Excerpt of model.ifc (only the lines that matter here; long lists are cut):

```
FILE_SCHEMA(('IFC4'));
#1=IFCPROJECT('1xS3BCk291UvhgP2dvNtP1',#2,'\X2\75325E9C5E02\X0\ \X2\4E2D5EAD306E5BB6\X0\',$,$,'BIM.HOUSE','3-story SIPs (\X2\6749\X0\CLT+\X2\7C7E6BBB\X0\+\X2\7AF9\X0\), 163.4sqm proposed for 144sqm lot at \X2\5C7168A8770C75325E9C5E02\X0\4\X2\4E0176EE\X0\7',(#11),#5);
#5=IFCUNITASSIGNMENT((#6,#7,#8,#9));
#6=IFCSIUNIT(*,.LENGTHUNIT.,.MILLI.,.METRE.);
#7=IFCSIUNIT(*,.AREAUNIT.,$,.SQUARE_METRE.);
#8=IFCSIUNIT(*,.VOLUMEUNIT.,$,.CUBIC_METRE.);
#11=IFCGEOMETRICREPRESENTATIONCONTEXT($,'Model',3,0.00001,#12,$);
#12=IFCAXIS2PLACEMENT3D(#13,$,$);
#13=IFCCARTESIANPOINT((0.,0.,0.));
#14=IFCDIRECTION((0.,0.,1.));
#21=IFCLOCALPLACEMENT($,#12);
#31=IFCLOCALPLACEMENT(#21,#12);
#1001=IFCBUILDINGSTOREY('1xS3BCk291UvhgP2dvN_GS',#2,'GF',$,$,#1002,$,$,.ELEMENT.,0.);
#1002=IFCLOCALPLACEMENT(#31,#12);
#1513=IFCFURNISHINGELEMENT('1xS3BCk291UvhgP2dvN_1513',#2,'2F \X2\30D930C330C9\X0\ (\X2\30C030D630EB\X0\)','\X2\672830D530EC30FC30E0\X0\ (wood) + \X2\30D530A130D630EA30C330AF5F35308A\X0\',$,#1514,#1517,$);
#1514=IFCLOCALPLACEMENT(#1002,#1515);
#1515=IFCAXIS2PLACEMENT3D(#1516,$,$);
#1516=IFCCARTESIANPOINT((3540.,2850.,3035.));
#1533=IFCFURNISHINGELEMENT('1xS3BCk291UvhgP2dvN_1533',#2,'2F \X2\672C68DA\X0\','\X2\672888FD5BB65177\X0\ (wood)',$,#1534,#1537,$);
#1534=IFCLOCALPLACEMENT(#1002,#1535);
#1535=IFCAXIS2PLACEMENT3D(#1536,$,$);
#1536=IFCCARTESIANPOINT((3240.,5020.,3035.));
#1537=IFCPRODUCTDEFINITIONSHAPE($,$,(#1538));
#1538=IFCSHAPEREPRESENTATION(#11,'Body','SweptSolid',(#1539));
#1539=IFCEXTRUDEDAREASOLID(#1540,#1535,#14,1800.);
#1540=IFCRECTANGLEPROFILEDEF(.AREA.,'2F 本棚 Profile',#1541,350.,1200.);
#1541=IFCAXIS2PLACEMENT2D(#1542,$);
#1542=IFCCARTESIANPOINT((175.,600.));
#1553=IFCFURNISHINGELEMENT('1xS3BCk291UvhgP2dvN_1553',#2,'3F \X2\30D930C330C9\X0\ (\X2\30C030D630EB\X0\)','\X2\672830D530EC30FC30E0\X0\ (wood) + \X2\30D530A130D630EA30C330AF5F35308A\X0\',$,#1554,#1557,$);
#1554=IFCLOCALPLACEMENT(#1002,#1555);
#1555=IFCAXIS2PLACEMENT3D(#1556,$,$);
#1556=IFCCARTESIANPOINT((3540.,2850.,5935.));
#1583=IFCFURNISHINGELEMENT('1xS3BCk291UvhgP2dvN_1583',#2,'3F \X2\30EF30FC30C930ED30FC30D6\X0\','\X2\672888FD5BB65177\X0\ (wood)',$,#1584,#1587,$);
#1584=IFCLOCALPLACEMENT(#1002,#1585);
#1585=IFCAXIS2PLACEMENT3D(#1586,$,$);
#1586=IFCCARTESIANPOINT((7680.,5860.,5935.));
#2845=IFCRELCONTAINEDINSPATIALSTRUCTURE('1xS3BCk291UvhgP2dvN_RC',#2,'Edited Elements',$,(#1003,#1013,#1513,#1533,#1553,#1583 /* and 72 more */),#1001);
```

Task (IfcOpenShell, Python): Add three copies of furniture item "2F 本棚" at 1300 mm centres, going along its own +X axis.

```python
import ifcopenshell
import ifcopenshell.api.geometry
import ifcopenshell.api.root
import ifcopenshell.util.element
import ifcopenshell.util.placement
import ifcopenshell.util.unit

model = ifcopenshell.open("model.ifc")
unit_scale = ifcopenshell.util.unit.calculate_unit_scale(model)


def reuse_history(source, copy):
    """copy_class also copies each property set's owner history, people and application; keep the originals."""
    for rel in copy.IsDefinedBy:
        if rel.is_a("IfcRelDefinesByProperties") and (history := rel.RelatingPropertyDefinition.OwnerHistory):
            rel.RelatingPropertyDefinition.OwnerHistory = source.OwnerHistory
            ifcopenshell.util.element.remove_deep2(model, history)


source = model.by_id(1533)
base = ifcopenshell.util.placement.get_local_placement(source.ObjectPlacement)
step = base[:3, 0] * 1.3 / unit_scale

for i in range(1, 4):
    copy = ifcopenshell.api.root.copy_class(model, product=source)
    copy.Representation = ifcopenshell.util.element.copy_deep(
        model, source.Representation, exclude=["IfcGeometricRepresentationContext", "IfcRepresentationMap"]
    )
    reuse_history(source, copy)
    matrix = base.copy()
    matrix[:3, 3] += i * step
    print("added at", matrix[:3, 3].round(3) + 0.0)
    ifcopenshell.api.geometry.edit_object_placement(model, product=copy, matrix=matrix, is_si=False)

model.write("model-out.ifc")
```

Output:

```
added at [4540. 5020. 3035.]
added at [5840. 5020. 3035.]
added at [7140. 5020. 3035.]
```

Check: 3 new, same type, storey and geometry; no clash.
